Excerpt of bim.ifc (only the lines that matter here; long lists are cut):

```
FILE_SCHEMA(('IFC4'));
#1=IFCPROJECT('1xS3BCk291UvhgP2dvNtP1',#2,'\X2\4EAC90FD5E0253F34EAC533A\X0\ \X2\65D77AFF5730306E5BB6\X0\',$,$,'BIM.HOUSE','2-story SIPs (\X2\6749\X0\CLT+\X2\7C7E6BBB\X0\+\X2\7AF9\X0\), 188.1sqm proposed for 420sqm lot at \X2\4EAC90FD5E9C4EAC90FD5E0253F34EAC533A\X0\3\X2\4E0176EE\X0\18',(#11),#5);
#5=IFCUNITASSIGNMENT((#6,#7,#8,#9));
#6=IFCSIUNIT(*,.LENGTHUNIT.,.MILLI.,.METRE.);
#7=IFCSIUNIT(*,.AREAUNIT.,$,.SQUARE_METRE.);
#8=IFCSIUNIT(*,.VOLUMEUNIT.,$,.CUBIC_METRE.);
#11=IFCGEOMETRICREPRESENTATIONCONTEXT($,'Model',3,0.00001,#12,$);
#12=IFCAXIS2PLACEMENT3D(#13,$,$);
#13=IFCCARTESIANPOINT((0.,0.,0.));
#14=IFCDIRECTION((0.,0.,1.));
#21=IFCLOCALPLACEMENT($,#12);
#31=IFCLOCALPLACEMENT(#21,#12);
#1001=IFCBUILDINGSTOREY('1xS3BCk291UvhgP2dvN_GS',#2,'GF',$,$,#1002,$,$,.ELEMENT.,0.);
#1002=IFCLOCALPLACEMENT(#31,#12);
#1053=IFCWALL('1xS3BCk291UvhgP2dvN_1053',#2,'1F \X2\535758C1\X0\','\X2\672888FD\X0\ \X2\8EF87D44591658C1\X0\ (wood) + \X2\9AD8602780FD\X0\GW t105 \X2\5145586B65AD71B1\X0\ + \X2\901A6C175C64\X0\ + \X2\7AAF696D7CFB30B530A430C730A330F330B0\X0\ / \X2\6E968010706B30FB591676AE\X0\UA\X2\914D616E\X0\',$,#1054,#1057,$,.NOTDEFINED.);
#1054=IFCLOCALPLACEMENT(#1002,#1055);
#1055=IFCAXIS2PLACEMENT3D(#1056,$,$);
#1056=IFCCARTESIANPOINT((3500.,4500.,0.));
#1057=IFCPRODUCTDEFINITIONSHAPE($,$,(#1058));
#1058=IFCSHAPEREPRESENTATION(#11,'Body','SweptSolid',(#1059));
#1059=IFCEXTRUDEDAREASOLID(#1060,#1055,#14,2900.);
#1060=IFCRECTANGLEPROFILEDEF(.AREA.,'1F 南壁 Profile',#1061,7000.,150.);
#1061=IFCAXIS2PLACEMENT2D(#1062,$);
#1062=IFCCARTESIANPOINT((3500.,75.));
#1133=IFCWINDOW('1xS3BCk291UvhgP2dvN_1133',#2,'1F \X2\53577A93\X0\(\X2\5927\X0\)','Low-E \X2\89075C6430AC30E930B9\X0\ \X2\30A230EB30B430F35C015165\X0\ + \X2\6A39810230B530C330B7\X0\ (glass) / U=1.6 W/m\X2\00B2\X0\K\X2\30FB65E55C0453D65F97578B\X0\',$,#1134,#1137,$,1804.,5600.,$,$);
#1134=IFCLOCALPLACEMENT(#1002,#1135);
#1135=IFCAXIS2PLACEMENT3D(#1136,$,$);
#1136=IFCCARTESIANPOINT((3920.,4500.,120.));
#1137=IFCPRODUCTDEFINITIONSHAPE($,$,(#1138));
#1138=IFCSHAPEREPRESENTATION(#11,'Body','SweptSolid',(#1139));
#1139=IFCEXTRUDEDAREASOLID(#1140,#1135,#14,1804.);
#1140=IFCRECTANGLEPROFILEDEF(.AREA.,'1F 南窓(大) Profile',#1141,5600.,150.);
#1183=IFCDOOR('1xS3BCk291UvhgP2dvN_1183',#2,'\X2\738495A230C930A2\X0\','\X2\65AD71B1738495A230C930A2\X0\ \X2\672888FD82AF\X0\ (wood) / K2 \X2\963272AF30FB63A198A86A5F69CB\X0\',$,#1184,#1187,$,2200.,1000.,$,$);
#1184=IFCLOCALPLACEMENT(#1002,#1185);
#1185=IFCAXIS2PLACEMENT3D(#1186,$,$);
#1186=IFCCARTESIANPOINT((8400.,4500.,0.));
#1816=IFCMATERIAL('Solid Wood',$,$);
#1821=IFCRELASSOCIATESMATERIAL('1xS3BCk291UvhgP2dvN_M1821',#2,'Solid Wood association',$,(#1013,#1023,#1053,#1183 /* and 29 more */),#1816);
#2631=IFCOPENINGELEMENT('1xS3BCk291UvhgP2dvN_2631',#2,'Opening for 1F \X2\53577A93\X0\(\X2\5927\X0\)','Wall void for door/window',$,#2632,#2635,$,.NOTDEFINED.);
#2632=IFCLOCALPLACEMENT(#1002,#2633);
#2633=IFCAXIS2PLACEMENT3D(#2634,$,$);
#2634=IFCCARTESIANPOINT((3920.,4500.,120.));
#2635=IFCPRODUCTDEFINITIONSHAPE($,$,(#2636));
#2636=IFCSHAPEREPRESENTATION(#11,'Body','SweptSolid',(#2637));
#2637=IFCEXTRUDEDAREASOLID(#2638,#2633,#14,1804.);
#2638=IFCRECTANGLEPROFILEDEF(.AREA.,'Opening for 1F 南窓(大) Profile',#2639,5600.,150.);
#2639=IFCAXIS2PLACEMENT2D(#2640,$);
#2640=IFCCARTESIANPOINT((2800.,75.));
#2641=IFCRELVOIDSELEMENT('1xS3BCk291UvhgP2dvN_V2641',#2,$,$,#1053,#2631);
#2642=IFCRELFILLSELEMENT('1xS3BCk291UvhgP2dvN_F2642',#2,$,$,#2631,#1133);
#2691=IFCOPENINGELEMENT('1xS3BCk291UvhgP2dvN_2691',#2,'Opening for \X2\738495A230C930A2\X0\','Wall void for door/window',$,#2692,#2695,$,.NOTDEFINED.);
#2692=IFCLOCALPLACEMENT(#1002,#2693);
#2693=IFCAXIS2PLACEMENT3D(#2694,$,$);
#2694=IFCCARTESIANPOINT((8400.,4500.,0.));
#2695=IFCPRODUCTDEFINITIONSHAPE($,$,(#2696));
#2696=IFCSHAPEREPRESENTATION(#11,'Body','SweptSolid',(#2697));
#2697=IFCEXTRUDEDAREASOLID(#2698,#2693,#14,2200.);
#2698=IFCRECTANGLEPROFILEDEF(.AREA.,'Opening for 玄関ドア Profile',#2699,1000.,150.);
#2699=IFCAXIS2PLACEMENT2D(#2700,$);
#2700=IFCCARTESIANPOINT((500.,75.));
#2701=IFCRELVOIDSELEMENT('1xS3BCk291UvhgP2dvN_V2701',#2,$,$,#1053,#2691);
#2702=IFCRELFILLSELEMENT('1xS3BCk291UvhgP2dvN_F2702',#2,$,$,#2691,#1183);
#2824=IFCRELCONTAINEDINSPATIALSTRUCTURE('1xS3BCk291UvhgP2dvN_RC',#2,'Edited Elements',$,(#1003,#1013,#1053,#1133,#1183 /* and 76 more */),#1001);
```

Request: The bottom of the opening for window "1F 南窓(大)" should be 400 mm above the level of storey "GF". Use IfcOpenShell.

```python
import numpy as np
import ifcopenshell
import ifcopenshell.api.geometry
import ifcopenshell.geom
import ifcopenshell.util.element
import ifcopenshell.util.placement
import ifcopenshell.util.shape
import ifcopenshell.util.unit

model = ifcopenshell.open("bim.ifc")
unit_scale = ifcopenshell.util.unit.calculate_unit_scale(model)

window = model.by_guid("1xS3BCk291UvhgP2dvN_1133")
opening = window.FillsVoids[0].RelatingOpeningElement
storey = ifcopenshell.util.element.get_container(window, ifc_class="IfcBuildingStorey")
level = ifcopenshell.util.placement.get_local_placement(storey.ObjectPlacement)[2, 3]

# The opening's origin need not be at the sill, so measure its lowest point.
shape = ifcopenshell.geom.create_shape(ifcopenshell.geom.settings(), opening)
bottom = ifcopenshell.util.shape.get_shape_bottom_elevation(shape, shape.geometry) / unit_scale
dz = level + 0.4 / unit_scale - bottom

shift = np.array([0.0, 0.0, dz])
# The window is not placed relative to its opening, so move both.
for product in (opening, window):
    matrix = ifcopenshell.util.placement.get_local_placement(product.ObjectPlacement)
    matrix[:3, 3] += shift
    ifcopenshell.api.geometry.edit_object_placement(model, product=product, matrix=matrix, is_si=False)

print(f"moved by {dz * unit_scale:+.3f} m")

model.write("bim-out.ifc")
```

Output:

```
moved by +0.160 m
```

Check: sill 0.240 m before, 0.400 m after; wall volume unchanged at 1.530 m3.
